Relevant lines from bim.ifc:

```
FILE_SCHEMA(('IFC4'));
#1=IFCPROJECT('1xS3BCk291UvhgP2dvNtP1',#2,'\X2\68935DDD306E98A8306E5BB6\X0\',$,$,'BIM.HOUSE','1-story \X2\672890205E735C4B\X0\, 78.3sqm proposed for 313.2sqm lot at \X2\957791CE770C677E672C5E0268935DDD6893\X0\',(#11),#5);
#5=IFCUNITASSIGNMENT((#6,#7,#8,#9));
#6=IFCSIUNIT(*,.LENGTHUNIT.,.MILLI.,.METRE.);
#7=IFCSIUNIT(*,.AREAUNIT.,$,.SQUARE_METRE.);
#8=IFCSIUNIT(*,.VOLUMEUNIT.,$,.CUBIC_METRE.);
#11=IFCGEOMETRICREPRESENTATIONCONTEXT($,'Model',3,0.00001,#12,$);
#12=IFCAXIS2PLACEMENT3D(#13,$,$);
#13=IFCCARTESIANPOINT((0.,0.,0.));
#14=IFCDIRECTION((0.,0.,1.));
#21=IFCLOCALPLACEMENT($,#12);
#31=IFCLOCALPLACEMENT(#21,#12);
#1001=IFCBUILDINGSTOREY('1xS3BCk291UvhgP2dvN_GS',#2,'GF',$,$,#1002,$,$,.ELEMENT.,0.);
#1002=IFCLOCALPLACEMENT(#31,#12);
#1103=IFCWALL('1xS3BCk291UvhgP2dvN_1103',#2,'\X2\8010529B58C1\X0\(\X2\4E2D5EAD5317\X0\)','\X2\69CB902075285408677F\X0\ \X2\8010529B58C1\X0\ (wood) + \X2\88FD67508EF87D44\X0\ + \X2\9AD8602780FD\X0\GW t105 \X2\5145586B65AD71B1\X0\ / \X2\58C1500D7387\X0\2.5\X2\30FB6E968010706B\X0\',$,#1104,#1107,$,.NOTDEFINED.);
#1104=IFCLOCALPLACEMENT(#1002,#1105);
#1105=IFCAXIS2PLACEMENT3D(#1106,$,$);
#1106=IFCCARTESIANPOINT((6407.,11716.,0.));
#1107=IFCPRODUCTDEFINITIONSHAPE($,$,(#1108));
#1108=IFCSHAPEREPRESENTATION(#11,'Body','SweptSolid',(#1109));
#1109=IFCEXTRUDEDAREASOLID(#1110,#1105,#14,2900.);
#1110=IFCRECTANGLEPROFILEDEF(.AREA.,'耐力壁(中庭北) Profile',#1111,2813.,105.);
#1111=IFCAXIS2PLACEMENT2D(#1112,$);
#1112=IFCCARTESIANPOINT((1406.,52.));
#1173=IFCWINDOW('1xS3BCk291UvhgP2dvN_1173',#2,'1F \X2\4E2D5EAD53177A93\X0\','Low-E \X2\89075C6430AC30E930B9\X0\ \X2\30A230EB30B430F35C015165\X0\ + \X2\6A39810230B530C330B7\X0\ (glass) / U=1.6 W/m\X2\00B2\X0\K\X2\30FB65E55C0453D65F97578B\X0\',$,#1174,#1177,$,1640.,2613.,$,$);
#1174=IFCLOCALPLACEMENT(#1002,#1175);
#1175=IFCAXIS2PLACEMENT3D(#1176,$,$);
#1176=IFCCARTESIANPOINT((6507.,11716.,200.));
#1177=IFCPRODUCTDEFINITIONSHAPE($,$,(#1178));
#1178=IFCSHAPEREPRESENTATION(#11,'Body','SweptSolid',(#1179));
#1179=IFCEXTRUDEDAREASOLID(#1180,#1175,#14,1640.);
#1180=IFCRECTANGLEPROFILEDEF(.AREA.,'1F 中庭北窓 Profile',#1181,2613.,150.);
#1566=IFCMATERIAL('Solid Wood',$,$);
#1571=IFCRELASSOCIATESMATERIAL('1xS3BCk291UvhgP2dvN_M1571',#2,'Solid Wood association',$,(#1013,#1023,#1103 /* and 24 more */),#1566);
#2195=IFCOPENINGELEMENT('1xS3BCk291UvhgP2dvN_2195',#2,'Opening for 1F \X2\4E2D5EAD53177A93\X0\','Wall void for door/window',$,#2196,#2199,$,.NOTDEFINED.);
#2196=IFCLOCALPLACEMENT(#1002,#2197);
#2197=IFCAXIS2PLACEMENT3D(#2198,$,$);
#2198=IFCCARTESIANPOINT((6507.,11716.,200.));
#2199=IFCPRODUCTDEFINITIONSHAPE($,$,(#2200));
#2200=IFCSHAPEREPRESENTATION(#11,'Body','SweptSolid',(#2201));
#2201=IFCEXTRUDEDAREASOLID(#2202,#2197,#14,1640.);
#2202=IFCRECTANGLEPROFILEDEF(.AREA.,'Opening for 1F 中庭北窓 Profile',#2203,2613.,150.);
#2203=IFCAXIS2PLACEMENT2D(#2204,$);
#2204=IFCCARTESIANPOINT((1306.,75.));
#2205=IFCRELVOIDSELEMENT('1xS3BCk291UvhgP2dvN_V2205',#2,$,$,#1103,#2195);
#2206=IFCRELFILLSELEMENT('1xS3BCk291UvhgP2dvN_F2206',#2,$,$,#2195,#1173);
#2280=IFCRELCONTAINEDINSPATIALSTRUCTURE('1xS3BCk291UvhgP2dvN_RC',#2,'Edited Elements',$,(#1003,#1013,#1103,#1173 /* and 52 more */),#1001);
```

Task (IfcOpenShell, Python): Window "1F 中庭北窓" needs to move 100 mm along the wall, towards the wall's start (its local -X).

```python
import ifcopenshell
import ifcopenshell.api.geometry
import ifcopenshell.util.placement
import ifcopenshell.util.unit

model = ifcopenshell.open("bim.ifc")
unit_scale = ifcopenshell.util.unit.calculate_unit_scale(model)

window = model.by_guid("1xS3BCk291UvhgP2dvN_1173")
opening = window.FillsVoids[0].RelatingOpeningElement
wall = opening.VoidsElements[0].RelatingBuildingElement

wall_matrix = ifcopenshell.util.placement.get_local_placement(wall.ObjectPlacement)
shift = wall_matrix[:3, 0] * -0.1 / unit_scale
before = ifcopenshell.util.placement.get_local_placement(window.ObjectPlacement)[:3, 3].copy()

# The window is not placed relative to its opening, so move both.
for product in (opening, window):
    matrix = ifcopenshell.util.placement.get_local_placement(product.ObjectPlacement)
    matrix[:3, 3] += shift
    ifcopenshell.api.geometry.edit_object_placement(model, product=product, matrix=matrix, is_si=False)

after = ifcopenshell.util.placement.get_local_placement(window.ObjectPlacement)[:3, 3]
print("window moved by", (after - before).round(3) + 0.0)

model.write("bim_rev.ifc")
```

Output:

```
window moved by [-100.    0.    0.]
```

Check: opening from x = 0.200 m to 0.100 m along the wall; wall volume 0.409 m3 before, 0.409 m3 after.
